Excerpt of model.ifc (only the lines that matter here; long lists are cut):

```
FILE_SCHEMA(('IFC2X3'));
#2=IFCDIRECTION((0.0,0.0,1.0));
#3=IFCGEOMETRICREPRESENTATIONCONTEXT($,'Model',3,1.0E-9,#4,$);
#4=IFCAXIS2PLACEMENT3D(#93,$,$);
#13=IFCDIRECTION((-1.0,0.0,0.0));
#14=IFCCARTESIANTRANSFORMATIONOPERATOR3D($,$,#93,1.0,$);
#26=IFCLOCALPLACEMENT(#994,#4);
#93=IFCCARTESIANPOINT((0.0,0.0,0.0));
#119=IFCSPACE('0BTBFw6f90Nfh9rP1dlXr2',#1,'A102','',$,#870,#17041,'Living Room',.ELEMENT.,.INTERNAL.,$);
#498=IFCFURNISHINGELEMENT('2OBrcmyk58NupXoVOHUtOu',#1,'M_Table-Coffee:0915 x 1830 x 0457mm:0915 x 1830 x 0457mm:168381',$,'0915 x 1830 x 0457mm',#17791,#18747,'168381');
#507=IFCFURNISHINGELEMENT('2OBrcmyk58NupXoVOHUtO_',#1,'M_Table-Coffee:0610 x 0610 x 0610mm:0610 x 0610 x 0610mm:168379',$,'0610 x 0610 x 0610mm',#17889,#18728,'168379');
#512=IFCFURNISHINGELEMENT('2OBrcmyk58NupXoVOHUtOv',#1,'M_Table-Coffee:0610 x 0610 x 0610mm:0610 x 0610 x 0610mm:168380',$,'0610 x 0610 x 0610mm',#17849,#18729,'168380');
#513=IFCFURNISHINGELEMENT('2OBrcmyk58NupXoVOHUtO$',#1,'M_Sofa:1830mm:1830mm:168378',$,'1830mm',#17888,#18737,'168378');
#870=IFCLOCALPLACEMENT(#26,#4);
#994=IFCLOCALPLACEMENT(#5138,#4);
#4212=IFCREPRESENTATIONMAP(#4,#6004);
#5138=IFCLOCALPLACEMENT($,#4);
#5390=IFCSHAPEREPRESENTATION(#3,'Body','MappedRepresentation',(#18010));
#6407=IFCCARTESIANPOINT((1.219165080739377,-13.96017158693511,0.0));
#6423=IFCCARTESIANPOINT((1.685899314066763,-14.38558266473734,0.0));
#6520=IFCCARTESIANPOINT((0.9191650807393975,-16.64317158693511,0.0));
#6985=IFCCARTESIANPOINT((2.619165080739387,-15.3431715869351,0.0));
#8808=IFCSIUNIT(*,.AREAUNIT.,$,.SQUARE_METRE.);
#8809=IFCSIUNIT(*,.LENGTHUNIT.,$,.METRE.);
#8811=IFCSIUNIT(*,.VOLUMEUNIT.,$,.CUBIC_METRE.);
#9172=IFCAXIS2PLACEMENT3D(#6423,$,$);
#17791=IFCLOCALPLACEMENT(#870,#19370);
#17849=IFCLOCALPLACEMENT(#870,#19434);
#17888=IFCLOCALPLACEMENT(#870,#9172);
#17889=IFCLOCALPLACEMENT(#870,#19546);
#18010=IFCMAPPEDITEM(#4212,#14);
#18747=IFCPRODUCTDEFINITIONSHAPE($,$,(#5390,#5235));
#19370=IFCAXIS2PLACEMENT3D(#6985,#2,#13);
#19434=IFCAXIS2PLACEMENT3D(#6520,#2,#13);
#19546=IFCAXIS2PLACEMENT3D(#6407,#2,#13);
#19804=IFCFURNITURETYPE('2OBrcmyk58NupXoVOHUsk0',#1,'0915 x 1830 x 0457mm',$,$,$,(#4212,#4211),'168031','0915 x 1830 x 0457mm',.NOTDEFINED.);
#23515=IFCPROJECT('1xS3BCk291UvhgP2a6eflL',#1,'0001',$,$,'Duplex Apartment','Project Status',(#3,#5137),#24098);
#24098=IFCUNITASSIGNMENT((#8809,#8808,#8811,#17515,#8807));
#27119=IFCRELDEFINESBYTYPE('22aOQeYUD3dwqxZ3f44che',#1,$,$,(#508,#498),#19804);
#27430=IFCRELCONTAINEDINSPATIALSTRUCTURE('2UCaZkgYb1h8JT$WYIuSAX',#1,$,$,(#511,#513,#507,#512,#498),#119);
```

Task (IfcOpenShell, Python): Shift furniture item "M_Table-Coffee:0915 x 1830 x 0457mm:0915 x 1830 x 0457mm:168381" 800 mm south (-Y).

```python
import ifcopenshell
import ifcopenshell.api.geometry
import ifcopenshell.util.placement
import ifcopenshell.util.unit

model = ifcopenshell.open("model.ifc")
unit_scale = ifcopenshell.util.unit.calculate_unit_scale(model)

item = model.by_guid("2OBrcmyk58NupXoVOHUtOu")
matrix = ifcopenshell.util.placement.get_local_placement(item.ObjectPlacement)
matrix[1, 3] -= 0.8 / unit_scale
ifcopenshell.api.geometry.edit_object_placement(model, product=item, matrix=matrix, is_si=False)

print(ifcopenshell.util.placement.get_local_placement(item.ObjectPlacement).round(3) + 0.0)

model.write("model_edited.ifc")
```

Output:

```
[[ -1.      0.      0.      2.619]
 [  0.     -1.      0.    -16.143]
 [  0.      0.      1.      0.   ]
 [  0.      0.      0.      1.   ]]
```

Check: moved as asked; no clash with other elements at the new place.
